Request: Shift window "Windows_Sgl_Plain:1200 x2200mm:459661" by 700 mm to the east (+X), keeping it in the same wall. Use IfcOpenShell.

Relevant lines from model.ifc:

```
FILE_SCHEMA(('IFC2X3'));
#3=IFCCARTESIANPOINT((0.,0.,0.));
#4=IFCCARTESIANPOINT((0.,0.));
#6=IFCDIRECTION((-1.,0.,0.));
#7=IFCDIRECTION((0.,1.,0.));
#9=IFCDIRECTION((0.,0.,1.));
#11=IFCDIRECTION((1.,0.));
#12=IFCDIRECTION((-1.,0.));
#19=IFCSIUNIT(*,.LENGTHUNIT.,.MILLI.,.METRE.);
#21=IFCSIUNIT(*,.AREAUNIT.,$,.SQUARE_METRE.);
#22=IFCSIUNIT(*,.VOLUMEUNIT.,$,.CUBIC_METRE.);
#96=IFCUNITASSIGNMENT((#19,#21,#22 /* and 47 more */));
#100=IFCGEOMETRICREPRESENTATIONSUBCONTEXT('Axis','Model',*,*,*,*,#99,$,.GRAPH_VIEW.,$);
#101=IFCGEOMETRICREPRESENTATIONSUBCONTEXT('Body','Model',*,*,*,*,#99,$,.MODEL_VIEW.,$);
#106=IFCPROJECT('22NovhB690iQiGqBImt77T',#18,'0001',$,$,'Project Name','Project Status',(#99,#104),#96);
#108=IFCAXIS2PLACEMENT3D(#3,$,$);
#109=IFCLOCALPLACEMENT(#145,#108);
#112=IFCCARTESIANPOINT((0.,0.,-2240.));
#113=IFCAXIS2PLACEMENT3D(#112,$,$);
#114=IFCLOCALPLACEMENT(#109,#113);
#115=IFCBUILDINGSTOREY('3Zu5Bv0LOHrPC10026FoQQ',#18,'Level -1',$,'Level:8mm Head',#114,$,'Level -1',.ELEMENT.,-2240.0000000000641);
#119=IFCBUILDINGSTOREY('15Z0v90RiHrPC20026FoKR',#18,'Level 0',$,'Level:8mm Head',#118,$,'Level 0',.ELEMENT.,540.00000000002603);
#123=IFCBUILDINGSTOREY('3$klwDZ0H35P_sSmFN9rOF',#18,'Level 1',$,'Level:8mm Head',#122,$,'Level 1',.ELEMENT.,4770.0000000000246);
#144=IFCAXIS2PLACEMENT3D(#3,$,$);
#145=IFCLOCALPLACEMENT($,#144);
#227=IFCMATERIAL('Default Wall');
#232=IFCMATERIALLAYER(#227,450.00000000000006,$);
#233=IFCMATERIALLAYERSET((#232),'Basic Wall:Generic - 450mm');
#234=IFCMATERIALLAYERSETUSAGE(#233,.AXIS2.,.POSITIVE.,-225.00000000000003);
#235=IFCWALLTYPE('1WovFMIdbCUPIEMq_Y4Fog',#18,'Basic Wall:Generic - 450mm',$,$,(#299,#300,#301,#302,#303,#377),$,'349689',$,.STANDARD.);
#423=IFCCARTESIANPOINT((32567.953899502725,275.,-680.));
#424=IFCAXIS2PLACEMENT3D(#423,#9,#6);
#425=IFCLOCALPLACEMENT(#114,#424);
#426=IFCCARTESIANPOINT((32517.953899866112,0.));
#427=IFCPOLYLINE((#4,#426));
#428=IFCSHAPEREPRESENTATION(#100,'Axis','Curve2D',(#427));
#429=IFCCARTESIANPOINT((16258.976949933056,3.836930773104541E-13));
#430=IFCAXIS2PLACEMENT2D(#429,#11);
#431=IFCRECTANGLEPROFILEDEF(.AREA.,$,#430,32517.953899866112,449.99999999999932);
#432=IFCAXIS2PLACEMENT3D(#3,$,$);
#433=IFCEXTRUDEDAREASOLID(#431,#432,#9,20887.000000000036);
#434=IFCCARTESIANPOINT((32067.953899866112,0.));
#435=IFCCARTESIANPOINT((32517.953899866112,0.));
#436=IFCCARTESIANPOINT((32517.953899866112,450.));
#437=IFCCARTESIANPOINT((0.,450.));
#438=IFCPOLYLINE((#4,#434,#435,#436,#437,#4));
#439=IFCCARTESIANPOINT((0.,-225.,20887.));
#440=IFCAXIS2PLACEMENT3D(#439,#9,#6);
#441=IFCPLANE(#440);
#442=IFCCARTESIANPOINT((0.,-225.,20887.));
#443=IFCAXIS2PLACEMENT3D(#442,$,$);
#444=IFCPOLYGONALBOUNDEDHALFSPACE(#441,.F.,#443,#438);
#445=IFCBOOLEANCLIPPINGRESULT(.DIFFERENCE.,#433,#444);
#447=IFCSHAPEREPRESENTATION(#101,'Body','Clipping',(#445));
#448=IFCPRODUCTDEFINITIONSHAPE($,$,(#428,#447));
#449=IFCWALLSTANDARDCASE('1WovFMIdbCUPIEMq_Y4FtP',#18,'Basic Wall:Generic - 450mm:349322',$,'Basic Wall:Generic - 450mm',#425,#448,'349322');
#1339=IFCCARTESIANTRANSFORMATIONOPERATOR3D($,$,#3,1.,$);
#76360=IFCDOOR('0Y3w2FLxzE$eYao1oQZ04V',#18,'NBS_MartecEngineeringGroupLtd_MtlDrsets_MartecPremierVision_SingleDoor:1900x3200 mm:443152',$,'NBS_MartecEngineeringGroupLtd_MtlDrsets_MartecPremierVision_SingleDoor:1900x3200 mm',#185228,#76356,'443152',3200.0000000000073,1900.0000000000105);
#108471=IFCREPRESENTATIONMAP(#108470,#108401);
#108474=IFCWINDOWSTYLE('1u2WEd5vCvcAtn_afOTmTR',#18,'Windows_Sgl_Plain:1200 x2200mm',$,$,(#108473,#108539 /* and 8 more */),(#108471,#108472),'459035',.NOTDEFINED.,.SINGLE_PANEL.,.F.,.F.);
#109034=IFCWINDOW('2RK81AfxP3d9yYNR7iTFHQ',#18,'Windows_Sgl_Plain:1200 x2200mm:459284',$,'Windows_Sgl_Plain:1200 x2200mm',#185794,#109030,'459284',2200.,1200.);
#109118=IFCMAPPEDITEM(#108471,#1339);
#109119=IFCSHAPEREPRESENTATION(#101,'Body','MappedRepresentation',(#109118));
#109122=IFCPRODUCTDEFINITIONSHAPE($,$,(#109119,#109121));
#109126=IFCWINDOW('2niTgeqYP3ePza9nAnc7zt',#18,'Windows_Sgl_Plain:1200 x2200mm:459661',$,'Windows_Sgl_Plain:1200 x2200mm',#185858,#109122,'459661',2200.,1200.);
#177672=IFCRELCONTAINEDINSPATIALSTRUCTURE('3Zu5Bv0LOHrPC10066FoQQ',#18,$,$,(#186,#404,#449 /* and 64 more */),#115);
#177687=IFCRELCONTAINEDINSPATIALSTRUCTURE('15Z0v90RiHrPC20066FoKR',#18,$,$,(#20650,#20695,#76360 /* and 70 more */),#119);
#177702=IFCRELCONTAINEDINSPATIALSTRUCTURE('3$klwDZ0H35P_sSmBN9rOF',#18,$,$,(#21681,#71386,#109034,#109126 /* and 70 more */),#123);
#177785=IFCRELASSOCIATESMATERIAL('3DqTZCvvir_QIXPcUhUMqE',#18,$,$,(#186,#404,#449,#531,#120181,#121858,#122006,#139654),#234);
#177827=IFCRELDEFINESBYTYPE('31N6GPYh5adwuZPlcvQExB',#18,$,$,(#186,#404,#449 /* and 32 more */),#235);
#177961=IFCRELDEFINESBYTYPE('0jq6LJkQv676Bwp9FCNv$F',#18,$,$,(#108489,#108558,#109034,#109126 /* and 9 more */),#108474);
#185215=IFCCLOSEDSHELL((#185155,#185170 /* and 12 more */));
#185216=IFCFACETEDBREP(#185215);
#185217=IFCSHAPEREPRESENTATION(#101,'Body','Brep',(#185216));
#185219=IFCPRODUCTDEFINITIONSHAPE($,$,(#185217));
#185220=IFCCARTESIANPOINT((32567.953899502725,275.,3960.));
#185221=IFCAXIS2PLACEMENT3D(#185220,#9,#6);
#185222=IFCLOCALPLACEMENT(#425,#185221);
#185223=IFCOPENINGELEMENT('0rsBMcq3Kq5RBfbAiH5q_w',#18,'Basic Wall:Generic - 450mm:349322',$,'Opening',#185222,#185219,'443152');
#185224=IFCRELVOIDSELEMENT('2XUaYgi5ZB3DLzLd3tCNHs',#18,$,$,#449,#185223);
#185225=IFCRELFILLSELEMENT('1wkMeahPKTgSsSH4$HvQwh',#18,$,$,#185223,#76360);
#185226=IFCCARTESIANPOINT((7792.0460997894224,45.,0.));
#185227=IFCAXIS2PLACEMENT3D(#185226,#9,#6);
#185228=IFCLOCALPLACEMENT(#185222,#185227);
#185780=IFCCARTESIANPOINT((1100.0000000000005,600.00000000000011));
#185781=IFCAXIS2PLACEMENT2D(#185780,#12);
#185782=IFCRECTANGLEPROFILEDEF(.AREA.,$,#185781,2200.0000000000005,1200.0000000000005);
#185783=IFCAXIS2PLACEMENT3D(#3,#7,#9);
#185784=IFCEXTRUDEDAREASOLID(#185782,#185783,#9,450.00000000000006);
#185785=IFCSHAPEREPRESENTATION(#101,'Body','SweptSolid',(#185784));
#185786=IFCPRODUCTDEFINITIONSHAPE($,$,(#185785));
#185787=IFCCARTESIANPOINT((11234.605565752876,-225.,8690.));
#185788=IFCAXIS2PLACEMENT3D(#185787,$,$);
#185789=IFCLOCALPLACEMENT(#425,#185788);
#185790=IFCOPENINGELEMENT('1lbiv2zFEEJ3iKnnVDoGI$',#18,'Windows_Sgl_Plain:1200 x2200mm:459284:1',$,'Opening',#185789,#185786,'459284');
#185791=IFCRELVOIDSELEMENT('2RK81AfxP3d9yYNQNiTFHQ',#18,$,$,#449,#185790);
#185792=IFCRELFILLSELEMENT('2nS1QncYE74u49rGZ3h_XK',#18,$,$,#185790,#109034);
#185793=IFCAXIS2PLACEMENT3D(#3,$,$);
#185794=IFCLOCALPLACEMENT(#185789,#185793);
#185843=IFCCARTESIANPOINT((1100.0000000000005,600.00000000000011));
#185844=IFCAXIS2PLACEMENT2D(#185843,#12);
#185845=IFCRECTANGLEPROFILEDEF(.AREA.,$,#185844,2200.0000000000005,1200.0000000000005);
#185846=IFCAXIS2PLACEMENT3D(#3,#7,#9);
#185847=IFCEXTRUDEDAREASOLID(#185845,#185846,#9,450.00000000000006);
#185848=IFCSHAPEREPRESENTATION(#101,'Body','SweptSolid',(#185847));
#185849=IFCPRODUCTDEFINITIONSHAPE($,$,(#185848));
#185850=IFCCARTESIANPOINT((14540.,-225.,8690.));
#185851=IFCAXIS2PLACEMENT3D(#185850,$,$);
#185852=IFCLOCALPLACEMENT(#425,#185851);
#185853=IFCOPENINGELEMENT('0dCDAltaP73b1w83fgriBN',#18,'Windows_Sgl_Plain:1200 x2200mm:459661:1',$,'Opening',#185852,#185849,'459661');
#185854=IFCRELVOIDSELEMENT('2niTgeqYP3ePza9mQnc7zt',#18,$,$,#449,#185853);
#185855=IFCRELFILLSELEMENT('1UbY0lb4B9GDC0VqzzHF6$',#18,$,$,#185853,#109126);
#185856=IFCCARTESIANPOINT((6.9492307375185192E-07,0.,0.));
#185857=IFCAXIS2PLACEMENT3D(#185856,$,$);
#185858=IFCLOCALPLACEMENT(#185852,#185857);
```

```python
import ifcopenshell
import ifcopenshell.api.geometry
import ifcopenshell.util.placement
import ifcopenshell.util.unit

model = ifcopenshell.open("model.ifc")
unit_scale = ifcopenshell.util.unit.calculate_unit_scale(model)

window = model.by_guid("2niTgeqYP3ePza9nAnc7zt")
opening = window.FillsVoids[0].RelatingOpeningElement
wall = opening.VoidsElements[0].RelatingBuildingElement

wall_matrix = ifcopenshell.util.placement.get_local_placement(wall.ObjectPlacement)
shift = wall_matrix[:3, 0] * -0.7 / unit_scale
before = ifcopenshell.util.placement.get_local_placement(window.ObjectPlacement)[:3, 3].copy()

# The window is placed relative to its opening, so it follows when the opening moves.
matrix = ifcopenshell.util.placement.get_local_placement(opening.ObjectPlacement)
matrix[:3, 3] += shift
ifcopenshell.api.geometry.edit_object_placement(
    model, product=opening, matrix=matrix, is_si=False, should_transform_children=True
)

after = ifcopenshell.util.placement.get_local_placement(window.ObjectPlacement)[:3, 3]
print("window moved by", (after - before).round(3) + 0.0)

model.write("model_edited.ifc")
```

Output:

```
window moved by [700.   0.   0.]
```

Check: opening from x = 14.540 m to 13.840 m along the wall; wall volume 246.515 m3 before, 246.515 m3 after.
